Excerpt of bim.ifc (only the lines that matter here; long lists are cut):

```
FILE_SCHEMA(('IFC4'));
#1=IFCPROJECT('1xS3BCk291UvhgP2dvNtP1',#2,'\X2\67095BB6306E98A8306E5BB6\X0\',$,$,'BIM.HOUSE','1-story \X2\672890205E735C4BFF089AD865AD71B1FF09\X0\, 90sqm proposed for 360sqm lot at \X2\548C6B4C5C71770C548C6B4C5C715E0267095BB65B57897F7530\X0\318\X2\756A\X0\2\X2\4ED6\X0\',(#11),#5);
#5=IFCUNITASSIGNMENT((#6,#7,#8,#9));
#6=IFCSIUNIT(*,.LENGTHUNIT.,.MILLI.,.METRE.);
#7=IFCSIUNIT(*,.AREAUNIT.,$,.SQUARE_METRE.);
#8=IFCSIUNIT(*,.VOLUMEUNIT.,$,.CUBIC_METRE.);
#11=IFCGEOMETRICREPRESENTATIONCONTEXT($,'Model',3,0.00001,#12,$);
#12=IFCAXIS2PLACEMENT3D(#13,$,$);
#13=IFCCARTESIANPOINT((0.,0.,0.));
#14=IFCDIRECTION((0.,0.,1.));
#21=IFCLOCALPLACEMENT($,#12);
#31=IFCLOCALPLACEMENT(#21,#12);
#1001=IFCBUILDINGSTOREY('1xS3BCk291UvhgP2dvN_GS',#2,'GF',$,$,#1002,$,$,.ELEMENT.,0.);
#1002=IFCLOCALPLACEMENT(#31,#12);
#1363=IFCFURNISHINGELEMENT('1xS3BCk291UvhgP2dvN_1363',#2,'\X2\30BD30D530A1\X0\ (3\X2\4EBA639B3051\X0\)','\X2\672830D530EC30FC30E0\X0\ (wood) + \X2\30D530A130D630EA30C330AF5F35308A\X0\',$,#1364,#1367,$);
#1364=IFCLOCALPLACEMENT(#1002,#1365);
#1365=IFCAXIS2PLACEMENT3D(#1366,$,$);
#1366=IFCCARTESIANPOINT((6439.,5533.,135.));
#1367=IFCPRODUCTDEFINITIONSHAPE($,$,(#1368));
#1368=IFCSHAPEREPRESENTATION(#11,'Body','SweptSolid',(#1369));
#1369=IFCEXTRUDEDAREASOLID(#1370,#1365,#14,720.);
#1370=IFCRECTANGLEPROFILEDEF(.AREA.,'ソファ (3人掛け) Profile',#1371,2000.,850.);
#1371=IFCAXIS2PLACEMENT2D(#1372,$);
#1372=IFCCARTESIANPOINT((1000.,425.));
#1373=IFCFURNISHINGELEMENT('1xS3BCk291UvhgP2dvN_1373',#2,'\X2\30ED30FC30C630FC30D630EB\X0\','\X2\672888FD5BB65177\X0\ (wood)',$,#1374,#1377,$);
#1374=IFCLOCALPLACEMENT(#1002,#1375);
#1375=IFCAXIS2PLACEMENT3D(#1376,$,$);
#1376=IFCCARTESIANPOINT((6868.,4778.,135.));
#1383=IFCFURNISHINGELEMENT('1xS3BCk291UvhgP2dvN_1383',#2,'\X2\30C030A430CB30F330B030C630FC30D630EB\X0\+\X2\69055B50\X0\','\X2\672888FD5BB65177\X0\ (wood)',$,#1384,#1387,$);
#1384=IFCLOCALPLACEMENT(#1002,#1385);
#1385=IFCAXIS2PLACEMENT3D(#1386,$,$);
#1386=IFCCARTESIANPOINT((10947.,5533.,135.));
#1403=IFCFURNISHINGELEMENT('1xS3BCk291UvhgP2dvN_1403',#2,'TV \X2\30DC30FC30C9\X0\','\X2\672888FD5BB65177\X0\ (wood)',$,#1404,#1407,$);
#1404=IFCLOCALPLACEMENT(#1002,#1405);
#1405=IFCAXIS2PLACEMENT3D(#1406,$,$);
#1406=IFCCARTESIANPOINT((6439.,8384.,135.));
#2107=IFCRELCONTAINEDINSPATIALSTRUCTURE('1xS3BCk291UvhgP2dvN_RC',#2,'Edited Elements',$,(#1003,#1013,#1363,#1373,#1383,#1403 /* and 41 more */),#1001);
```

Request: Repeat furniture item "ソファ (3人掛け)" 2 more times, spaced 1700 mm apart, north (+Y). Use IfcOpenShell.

```python
import numpy as np
import ifcopenshell
import ifcopenshell.api.geometry
import ifcopenshell.api.root
import ifcopenshell.util.element
import ifcopenshell.util.placement
import ifcopenshell.util.unit

model = ifcopenshell.open("bim.ifc")
unit_scale = ifcopenshell.util.unit.calculate_unit_scale(model)


def reuse_history(source, copy):
    """copy_class also copies each property set's owner history, people and application; keep the originals."""
    for rel in copy.IsDefinedBy:
        if rel.is_a("IfcRelDefinesByProperties") and (history := rel.RelatingPropertyDefinition.OwnerHistory):
            rel.RelatingPropertyDefinition.OwnerHistory = source.OwnerHistory
            ifcopenshell.util.element.remove_deep2(model, history)


source = model.by_id(1363)
base = ifcopenshell.util.placement.get_local_placement(source.ObjectPlacement)
step = np.array([0.0, 1.0, 0.0]) * 1.7 / unit_scale

for i in range(1, 3):
    copy = ifcopenshell.api.root.copy_class(model, product=source)
    copy.Representation = ifcopenshell.util.element.copy_deep(
        model, source.Representation, exclude=["IfcGeometricRepresentationContext", "IfcRepresentationMap"]
    )
    reuse_history(source, copy)
    matrix = base.copy()
    matrix[:3, 3] += i * step
    print("added at", matrix[:3, 3].round(3) + 0.0)
    ifcopenshell.api.geometry.edit_object_placement(model, product=copy, matrix=matrix, is_si=False)

model.write("bim_v2.ifc")
```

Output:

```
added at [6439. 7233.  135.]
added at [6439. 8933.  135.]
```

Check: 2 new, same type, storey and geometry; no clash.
